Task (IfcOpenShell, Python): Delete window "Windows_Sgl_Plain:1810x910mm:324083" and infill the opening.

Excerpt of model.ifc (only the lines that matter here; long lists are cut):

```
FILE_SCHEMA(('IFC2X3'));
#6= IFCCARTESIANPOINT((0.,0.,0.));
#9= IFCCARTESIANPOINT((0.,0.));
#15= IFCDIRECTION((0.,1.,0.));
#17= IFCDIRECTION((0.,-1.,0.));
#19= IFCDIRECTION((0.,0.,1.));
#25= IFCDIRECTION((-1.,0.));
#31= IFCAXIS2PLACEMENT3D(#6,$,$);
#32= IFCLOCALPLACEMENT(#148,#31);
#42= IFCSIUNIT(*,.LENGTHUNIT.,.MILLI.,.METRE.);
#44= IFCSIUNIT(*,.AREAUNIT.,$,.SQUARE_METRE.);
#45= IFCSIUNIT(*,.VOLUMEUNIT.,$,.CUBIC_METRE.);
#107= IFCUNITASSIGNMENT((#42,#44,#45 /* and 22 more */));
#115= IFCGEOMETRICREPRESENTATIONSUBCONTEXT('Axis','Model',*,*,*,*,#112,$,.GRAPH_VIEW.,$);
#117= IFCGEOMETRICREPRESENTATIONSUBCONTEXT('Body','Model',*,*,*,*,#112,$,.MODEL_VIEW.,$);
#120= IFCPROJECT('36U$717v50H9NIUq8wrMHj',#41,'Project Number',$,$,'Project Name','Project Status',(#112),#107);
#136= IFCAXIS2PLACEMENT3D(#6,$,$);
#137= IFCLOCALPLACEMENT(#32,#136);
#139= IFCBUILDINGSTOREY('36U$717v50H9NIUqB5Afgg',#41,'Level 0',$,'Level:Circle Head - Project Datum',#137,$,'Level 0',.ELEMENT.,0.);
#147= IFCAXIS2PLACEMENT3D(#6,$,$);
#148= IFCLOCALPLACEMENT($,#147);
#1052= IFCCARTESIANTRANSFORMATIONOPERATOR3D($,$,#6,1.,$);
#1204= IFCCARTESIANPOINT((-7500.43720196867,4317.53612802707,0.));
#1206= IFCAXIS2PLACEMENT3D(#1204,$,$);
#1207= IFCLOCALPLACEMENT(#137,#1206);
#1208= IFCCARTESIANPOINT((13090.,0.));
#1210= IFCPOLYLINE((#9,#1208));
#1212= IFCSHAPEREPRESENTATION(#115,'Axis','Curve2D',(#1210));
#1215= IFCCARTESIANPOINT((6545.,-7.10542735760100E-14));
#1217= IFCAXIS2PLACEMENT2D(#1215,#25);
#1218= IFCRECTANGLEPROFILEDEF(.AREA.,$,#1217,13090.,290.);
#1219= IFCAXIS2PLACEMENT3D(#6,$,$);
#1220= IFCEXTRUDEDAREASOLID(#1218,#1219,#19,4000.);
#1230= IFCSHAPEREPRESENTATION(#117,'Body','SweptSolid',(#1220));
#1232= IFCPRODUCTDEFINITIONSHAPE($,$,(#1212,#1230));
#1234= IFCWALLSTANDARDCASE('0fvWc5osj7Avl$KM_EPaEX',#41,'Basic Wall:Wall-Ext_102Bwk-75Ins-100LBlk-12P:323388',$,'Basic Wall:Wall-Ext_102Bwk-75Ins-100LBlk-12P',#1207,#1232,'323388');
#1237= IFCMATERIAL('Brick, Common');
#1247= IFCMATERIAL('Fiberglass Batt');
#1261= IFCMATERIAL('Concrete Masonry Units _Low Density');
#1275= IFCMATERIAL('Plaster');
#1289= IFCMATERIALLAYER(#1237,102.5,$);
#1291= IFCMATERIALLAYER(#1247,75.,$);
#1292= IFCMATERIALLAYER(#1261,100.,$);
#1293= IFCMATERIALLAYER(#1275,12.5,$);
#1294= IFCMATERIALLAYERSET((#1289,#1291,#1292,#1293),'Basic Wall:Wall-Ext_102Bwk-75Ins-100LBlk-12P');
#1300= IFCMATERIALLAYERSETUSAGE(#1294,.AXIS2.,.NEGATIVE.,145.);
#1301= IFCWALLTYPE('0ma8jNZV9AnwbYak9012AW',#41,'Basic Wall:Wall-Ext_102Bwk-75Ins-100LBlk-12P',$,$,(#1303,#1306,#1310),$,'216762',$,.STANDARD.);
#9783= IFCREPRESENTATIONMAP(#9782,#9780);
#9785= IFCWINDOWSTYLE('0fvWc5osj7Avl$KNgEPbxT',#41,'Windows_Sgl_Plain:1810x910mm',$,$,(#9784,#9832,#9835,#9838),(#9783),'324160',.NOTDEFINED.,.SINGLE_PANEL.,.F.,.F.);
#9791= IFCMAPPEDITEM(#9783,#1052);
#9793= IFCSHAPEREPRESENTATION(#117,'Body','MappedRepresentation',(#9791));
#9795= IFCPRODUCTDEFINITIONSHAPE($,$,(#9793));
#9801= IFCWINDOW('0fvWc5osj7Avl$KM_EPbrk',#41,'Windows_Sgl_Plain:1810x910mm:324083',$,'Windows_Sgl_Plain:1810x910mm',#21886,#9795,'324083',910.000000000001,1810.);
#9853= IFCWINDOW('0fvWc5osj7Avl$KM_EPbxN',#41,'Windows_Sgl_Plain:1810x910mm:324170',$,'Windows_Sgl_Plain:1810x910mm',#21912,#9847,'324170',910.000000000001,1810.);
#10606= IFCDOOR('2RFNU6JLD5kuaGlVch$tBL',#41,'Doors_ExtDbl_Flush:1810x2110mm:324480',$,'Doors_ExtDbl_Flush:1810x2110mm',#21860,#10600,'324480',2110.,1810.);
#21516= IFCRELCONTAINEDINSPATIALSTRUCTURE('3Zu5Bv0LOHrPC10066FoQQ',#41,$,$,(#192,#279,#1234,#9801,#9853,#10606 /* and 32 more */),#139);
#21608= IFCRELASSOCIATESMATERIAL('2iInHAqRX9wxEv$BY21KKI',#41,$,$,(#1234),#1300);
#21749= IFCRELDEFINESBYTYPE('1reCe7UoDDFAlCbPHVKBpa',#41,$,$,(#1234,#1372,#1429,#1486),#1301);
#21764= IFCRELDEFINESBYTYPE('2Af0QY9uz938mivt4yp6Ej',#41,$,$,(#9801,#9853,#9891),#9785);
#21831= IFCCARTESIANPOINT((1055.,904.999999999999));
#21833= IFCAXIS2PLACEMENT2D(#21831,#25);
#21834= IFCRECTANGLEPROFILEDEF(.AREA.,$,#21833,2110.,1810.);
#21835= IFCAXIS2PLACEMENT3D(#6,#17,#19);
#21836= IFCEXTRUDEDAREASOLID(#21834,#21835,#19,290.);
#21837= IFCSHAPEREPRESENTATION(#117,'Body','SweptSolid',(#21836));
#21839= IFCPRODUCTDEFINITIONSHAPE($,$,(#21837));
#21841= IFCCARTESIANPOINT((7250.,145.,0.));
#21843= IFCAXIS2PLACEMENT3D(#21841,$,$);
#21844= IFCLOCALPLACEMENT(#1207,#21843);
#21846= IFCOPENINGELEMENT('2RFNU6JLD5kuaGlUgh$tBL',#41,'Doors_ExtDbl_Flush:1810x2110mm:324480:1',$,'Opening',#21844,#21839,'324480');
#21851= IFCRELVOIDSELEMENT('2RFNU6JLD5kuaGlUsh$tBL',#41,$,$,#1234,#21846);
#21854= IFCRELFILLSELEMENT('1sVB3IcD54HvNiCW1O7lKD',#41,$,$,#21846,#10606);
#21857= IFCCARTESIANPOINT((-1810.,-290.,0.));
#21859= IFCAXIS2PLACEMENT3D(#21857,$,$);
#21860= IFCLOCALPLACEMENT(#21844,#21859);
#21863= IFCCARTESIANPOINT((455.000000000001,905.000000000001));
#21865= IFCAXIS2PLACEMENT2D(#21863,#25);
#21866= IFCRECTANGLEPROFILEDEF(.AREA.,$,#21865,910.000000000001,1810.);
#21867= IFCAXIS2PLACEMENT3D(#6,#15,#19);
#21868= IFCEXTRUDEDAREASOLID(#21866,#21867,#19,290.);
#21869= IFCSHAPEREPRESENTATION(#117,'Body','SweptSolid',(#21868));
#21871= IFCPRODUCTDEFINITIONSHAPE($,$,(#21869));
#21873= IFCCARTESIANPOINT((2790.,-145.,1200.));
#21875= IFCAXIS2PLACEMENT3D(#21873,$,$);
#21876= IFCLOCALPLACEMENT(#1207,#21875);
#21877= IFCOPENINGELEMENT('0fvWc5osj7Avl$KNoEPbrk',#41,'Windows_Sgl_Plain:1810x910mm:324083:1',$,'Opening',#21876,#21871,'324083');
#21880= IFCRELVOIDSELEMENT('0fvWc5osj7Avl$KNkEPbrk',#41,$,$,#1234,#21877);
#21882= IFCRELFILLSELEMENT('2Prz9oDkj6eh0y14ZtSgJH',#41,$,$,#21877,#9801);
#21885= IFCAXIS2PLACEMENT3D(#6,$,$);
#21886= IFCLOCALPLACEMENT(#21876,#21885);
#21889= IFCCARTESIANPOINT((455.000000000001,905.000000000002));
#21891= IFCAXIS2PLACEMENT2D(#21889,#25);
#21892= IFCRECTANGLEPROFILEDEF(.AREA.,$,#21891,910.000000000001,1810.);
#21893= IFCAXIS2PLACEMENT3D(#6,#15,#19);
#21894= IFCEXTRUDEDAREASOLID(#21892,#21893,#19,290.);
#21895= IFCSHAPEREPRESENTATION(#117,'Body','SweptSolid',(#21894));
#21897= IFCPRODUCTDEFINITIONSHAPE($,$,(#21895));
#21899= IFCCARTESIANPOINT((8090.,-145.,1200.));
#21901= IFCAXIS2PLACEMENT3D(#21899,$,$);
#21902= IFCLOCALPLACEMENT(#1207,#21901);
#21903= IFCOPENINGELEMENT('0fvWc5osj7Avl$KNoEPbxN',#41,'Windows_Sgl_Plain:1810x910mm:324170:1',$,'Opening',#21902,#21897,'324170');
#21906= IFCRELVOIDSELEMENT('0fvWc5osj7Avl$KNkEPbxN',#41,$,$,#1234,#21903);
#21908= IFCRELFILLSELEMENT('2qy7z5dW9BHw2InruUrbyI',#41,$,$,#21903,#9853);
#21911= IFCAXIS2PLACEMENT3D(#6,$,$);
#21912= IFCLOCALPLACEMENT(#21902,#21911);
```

```python
import ifcopenshell
import ifcopenshell.api.feature
import ifcopenshell.api.root
import ifcopenshell.geom
import ifcopenshell.util.shape

model = ifcopenshell.open("model.ifc")
settings = ifcopenshell.geom.settings()


def volume(element):
    """Net volume in cubic metres, openings subtracted."""
    shape = ifcopenshell.geom.create_shape(settings, element)
    return ifcopenshell.util.shape.get_volume(shape.geometry)


window = model.by_guid("0fvWc5osj7Avl$KM_EPbrk")
opening = window.FillsVoids[0].RelatingOpeningElement
wall = opening.VoidsElements[0].RelatingBuildingElement
before = volume(wall)

ifcopenshell.api.root.remove_product(model, product=window)
ifcopenshell.api.feature.remove_feature(model, feature=opening)

after = volume(wall)

print(f"wall volume {before:.3f} -> {after:.3f} m3")

model.write("model_updated.ifc")
```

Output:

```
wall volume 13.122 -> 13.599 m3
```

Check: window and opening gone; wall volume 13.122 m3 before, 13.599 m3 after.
